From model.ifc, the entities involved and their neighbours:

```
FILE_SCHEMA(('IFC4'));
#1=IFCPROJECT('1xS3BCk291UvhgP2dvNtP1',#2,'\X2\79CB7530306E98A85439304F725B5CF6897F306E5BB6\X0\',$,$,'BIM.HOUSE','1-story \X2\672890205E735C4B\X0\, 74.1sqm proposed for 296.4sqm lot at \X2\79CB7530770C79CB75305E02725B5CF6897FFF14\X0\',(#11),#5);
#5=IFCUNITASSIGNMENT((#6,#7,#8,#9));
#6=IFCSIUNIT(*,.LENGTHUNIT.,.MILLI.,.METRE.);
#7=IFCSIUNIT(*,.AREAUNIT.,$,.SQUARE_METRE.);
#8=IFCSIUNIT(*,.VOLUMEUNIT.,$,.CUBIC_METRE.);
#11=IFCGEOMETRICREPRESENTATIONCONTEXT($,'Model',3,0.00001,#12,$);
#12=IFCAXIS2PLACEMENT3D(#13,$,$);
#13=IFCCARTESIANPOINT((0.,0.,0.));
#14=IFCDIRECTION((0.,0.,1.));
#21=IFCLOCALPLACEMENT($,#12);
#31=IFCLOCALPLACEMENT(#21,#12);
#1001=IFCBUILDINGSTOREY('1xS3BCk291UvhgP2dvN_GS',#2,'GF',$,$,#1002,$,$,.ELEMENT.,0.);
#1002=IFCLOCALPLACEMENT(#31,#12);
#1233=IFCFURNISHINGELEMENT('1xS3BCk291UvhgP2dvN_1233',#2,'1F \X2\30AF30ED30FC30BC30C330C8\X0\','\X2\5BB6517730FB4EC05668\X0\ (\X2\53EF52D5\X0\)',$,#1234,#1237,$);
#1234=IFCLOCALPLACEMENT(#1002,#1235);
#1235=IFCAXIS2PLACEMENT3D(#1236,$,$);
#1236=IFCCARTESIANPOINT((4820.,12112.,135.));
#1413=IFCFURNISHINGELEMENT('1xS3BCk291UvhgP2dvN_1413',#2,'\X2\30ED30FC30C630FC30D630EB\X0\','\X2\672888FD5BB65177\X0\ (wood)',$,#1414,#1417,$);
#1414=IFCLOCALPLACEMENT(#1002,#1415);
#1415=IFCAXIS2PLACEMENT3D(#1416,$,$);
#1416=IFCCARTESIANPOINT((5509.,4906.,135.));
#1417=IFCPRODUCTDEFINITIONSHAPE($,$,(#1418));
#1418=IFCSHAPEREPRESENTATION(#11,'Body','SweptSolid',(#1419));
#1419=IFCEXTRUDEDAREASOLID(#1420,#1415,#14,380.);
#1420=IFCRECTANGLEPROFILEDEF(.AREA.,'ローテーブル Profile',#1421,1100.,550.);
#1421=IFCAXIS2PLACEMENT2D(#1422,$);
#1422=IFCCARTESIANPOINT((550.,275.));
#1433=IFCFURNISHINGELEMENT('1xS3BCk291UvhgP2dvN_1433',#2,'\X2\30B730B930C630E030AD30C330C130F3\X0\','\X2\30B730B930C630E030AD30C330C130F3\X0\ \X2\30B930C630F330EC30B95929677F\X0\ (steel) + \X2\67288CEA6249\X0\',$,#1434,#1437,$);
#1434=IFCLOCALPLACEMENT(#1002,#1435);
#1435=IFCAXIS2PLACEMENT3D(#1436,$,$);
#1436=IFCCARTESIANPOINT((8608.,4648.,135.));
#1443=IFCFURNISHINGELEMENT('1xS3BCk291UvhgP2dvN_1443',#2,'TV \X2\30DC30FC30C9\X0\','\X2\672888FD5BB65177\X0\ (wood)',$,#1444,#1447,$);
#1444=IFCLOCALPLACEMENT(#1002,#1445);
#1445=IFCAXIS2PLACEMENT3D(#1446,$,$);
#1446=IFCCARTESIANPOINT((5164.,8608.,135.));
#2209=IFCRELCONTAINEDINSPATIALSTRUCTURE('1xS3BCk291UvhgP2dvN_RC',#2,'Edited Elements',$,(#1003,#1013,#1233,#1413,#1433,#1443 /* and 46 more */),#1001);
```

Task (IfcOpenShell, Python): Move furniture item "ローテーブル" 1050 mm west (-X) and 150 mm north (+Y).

```python
import ifcopenshell
import ifcopenshell.api.geometry
import ifcopenshell.util.placement
import ifcopenshell.util.unit

model = ifcopenshell.open("model.ifc")
unit_scale = ifcopenshell.util.unit.calculate_unit_scale(model)

item = model.by_guid("1xS3BCk291UvhgP2dvN_1413")
matrix = ifcopenshell.util.placement.get_local_placement(item.ObjectPlacement)
matrix[0, 3] -= 1.05 / unit_scale
matrix[1, 3] += 0.15 / unit_scale
ifcopenshell.api.geometry.edit_object_placement(model, product=item, matrix=matrix, is_si=False)

print(ifcopenshell.util.placement.get_local_placement(item.ObjectPlacement).round(3) + 0.0)

model.write("model_edited.ifc")
```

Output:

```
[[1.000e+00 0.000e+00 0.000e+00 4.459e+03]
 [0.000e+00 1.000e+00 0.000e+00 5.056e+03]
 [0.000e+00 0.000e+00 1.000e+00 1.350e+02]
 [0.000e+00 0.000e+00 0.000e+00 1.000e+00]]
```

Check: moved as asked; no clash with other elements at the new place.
